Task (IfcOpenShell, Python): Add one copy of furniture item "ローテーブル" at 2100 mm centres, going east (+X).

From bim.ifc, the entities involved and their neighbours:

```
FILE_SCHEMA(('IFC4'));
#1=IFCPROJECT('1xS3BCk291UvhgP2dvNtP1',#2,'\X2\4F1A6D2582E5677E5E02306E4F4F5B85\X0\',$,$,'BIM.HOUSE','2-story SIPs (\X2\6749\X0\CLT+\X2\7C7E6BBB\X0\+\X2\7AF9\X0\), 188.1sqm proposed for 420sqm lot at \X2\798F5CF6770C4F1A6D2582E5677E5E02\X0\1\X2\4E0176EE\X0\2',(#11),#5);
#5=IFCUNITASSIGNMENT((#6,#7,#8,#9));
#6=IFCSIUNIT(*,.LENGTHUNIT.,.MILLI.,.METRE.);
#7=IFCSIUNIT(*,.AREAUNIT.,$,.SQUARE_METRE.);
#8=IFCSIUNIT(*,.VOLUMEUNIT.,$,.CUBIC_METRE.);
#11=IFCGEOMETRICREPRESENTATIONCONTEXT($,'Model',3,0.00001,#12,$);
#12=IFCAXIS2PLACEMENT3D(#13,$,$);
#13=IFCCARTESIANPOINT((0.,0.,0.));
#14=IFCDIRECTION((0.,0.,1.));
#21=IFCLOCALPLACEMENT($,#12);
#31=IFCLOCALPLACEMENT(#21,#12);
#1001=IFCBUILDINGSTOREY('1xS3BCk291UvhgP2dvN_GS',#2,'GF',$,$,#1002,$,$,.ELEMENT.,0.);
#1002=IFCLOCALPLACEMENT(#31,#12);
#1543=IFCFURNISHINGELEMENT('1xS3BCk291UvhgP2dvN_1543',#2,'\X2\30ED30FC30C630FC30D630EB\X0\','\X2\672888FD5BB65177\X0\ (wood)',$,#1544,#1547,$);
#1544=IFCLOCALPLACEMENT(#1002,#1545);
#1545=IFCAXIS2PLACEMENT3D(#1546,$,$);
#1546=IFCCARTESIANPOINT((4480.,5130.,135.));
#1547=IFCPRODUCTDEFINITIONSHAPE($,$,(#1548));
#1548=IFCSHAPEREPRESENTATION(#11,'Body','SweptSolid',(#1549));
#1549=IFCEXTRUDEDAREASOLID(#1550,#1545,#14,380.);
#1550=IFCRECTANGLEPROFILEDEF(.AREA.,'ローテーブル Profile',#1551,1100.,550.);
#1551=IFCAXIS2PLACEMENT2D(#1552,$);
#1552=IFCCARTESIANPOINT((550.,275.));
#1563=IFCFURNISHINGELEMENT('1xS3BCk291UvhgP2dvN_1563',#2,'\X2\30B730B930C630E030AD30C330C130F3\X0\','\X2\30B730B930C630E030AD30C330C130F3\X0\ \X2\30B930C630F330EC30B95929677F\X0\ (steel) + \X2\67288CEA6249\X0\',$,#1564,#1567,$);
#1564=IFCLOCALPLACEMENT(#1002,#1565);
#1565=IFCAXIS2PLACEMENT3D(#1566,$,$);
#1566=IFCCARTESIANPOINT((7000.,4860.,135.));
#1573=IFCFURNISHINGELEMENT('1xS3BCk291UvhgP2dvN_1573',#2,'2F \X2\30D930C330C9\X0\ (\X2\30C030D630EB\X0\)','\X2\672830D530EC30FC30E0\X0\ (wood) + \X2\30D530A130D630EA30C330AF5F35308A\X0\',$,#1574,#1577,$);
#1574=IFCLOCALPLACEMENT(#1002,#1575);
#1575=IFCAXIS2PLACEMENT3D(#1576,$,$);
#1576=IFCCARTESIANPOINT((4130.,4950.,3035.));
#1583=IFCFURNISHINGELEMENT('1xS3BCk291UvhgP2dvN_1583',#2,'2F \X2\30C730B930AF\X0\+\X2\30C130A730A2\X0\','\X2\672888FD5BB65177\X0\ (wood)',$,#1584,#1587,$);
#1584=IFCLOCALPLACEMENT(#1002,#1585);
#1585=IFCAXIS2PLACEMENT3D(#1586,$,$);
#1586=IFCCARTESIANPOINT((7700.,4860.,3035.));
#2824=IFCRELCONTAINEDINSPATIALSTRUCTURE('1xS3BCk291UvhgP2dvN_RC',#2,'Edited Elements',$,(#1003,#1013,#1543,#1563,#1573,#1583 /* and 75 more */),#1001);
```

```python
import numpy as np
import ifcopenshell
import ifcopenshell.api.geometry
import ifcopenshell.api.root
import ifcopenshell.util.element
import ifcopenshell.util.placement

model = ifcopenshell.open("bim.ifc")


def reuse_history(source, copy):
    """copy_class also copies each property set's owner history, people and application; keep the originals."""
    for rel in copy.IsDefinedBy:
        if rel.is_a("IfcRelDefinesByProperties") and (history := rel.RelatingPropertyDefinition.OwnerHistory):
            rel.RelatingPropertyDefinition.OwnerHistory = source.OwnerHistory
            ifcopenshell.util.element.remove_deep2(model, history)


source = model.by_guid("1xS3BCk291UvhgP2dvN_1543")
base = ifcopenshell.util.placement.get_local_placement(source.ObjectPlacement)
step = np.array([1.0, 0.0, 0.0]) * 2100.0

for i in range(1, 2):
    copy = ifcopenshell.api.root.copy_class(model, product=source)
    copy.Representation = ifcopenshell.util.element.copy_deep(
        model, source.Representation, exclude=["IfcGeometricRepresentationContext", "IfcRepresentationMap"]
    )
    reuse_history(source, copy)
    matrix = base.copy()
    matrix[:3, 3] += i * step
    print("added at", matrix[:3, 3].round(3) + 0.0)
    ifcopenshell.api.geometry.edit_object_placement(model, product=copy, matrix=matrix, is_si=False)

model.write("bim_rev.ifc")
```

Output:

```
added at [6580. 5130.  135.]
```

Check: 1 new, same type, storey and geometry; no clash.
